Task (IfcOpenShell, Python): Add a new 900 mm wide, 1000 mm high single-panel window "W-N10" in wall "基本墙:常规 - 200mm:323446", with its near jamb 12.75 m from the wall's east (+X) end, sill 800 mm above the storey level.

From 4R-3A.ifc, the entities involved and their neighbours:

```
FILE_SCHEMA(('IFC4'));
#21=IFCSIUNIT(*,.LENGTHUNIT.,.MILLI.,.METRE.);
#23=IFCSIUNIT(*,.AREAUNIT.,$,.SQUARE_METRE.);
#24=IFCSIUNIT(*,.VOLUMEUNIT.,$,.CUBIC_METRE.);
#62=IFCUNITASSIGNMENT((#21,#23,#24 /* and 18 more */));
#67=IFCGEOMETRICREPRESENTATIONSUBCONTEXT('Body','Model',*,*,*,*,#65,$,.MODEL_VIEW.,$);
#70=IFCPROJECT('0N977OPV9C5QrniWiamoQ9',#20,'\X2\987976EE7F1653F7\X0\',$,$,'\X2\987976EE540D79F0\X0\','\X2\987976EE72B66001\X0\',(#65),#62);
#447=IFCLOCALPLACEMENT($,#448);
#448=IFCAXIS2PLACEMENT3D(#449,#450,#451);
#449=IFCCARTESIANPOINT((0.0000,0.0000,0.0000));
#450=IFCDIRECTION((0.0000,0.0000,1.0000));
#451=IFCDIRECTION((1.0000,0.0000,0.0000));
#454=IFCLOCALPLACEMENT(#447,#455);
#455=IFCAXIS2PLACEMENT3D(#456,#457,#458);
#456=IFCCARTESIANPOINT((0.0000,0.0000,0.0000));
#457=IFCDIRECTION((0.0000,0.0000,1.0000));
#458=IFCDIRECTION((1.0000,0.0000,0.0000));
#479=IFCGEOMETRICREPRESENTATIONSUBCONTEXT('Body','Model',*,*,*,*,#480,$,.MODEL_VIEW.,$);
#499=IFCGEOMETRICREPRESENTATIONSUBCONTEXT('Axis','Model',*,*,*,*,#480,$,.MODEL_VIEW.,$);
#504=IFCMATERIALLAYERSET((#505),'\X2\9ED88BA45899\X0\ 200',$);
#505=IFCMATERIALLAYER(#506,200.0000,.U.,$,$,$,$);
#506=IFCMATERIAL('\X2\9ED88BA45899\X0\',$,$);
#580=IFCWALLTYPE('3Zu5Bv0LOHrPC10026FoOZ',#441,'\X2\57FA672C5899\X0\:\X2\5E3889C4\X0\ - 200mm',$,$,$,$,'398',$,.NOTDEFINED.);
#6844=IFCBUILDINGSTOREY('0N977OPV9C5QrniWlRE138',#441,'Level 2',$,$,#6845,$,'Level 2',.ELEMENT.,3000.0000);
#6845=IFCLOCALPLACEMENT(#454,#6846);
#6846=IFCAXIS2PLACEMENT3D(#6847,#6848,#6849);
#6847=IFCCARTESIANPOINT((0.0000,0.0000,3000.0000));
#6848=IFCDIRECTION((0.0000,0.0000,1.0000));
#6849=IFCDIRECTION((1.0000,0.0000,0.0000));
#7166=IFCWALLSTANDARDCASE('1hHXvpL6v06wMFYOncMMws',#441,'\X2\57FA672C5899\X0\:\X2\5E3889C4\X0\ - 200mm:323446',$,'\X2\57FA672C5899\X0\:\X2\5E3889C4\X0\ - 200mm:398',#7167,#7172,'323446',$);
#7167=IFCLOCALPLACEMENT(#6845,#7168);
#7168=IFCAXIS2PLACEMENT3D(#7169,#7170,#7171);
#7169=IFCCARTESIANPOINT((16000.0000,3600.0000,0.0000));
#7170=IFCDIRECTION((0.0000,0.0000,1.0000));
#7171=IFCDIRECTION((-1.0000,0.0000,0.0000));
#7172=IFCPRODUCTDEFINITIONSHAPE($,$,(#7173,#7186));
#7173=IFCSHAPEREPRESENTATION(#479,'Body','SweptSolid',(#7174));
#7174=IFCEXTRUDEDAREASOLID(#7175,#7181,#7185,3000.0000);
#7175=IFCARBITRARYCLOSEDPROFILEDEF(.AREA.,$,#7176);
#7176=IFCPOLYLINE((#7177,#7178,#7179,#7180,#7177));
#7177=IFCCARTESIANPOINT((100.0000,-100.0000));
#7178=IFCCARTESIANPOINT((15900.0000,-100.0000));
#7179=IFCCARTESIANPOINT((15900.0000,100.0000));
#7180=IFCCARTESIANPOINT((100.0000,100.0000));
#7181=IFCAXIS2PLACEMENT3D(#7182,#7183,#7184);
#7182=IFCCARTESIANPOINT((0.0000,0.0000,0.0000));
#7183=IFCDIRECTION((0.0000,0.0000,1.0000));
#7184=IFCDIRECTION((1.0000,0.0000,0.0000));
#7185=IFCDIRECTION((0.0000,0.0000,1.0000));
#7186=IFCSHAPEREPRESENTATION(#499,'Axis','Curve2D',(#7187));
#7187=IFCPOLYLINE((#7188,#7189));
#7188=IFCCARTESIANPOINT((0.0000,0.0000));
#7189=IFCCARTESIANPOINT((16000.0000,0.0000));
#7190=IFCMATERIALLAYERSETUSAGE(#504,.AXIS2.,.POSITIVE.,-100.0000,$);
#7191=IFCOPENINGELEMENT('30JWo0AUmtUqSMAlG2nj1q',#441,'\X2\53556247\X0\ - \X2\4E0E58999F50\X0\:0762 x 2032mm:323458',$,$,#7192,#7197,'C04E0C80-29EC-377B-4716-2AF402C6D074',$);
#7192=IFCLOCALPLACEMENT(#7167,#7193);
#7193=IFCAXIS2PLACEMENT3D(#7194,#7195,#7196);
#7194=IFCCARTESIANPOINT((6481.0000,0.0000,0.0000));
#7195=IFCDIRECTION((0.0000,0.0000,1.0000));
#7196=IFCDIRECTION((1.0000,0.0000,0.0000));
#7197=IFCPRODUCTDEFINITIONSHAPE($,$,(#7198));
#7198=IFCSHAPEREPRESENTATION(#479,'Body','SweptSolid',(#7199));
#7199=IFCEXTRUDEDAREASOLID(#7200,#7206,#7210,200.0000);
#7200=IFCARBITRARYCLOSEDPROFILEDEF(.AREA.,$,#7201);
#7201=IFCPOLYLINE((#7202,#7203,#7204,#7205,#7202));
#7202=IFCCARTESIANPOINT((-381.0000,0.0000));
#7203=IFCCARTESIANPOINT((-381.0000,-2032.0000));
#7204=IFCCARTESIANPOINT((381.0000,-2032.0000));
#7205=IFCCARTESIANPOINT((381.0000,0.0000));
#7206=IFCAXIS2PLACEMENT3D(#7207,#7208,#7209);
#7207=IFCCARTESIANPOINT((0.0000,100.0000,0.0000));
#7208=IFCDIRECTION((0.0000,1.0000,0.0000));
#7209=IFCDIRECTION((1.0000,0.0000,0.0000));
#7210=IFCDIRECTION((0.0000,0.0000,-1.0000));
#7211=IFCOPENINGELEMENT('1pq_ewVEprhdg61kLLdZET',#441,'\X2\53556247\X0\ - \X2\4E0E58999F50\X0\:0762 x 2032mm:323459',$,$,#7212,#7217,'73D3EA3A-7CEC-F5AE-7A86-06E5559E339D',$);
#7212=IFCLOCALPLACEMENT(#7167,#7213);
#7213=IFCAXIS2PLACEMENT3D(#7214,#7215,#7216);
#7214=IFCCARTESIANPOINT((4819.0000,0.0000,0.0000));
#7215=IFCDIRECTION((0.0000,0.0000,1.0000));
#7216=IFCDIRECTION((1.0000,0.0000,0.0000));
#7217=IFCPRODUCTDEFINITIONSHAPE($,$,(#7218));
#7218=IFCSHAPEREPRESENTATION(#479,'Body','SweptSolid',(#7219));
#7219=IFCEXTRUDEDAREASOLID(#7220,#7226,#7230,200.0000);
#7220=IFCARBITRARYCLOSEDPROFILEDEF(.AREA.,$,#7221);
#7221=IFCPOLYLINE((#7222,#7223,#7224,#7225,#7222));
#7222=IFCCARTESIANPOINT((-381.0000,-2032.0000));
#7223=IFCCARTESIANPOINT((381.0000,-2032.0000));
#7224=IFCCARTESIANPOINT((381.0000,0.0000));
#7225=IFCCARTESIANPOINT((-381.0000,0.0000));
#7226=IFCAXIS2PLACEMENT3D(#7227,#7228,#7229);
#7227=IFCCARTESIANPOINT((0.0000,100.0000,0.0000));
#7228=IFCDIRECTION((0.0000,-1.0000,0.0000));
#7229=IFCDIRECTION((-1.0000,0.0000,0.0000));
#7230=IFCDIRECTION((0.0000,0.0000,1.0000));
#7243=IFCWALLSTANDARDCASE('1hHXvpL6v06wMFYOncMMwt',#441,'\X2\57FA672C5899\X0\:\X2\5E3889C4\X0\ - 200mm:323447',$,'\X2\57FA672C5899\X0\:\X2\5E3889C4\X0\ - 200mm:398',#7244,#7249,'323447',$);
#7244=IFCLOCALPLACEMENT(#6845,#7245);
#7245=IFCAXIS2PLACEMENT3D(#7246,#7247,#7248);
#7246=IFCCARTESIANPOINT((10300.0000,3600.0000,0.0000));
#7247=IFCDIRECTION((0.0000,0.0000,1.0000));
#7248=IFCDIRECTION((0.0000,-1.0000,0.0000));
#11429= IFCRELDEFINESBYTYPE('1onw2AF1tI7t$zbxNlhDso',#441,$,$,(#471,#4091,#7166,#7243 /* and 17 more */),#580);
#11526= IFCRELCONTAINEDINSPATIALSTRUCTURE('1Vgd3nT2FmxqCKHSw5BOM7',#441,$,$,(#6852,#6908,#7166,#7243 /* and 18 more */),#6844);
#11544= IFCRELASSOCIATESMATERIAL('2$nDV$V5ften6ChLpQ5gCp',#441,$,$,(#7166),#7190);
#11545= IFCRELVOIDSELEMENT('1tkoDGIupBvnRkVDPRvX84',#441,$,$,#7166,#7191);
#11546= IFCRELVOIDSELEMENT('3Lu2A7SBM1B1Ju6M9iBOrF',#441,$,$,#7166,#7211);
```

```python
import numpy as np
import ifcopenshell
import ifcopenshell.api.feature
import ifcopenshell.api.geometry
import ifcopenshell.api.root
import ifcopenshell.api.spatial
import ifcopenshell.geom
import ifcopenshell.util.element
import ifcopenshell.util.placement
import ifcopenshell.util.representation
import ifcopenshell.util.shape
import ifcopenshell.util.unit

model = ifcopenshell.open("4R-3A.ifc")
unit_scale = ifcopenshell.util.unit.calculate_unit_scale(model)
settings = ifcopenshell.geom.settings()


def volume(element):
    """Net volume in cubic metres, openings subtracted."""
    shape = ifcopenshell.geom.create_shape(settings, element)
    return ifcopenshell.util.shape.get_volume(shape.geometry)


wall = model.by_guid("1hHXvpL6v06wMFYOncMMws")
storey = ifcopenshell.util.element.get_container(wall, ifc_class="IfcBuildingStorey")
context = ifcopenshell.util.representation.get_context(model, "Model", "Body", "MODEL_VIEW")
before = volume(wall)

width, height, from_end, sill = 0.9, 1, 12.75, 0.8  # metres

# The wall runs along its own X axis, and the end named is its -X end.
wall_shape = ifcopenshell.geom.create_shape(settings, wall)
x, y, z = ifcopenshell.util.shape.get_vertices(wall_shape.geometry).T
start = x.min() + from_end
face, thickness = float(y.min()), float(y.max() - y.min())
wall_matrix = ifcopenshell.util.placement.get_local_placement(wall.ObjectPlacement)
level = ifcopenshell.util.placement.get_local_placement(storey.ObjectPlacement)[2, 3]


def in_wall(x, y):
    """Placement at x, y metres in the wall's axes, at sill height."""
    matrix = wall_matrix.copy()
    matrix[:, 3] = wall_matrix @ np.array([x / unit_scale, y / unit_scale, 0.0, 1.0])
    matrix[2, 3] = level + sill / unit_scale
    return matrix


# Opening: a box that overshoots both wall faces by 50 mm.
opening = ifcopenshell.api.root.create_entity(model, ifc_class="IfcOpeningElement", predefined_type="OPENING")
box = ifcopenshell.api.geometry.add_wall_representation(
    model, context=context, length=width, height=height, thickness=thickness + 0.1
)
ifcopenshell.api.geometry.assign_representation(model, product=opening, representation=box)
ifcopenshell.api.geometry.edit_object_placement(model, product=opening, matrix=in_wall(start, face - 0.05), is_si=False)
ifcopenshell.api.feature.add_feature(model, feature=opening, element=wall)

window = ifcopenshell.api.root.create_entity(model, ifc_class="IfcWindow", name="W-N10", predefined_type="WINDOW")
window.OverallWidth, window.OverallHeight = width / unit_scale, height / unit_scale
window.PartitioningType = "SINGLE_PANEL"
body = ifcopenshell.api.geometry.add_window_representation(
    model,
    context=context,
    overall_width=window.OverallWidth,
    overall_height=window.OverallHeight,
    partition_type="SINGLE_PANEL",
)
ifcopenshell.api.geometry.assign_representation(model, product=window, representation=body)
ifcopenshell.api.spatial.assign_container(model, products=[window], relating_structure=storey)
ifcopenshell.api.feature.add_filling(model, opening=opening, element=window)

# Centre the window in the wall's thickness.
ifcopenshell.api.geometry.edit_object_placement(model, product=window, matrix=in_wall(start, face), is_si=False)
window_shape = ifcopenshell.geom.create_shape(settings, window)
depth = ifcopenshell.util.shape.get_vertices(window_shape.geometry)[:, 1]
offset = face + thickness / 2 - (depth.min() + depth.max()) / 2
ifcopenshell.api.geometry.edit_object_placement(model, product=window, matrix=in_wall(start, offset), is_si=False)

after = volume(wall)

print(f"wall volume {before:.3f} -> {after:.3f} m3")

model.write("4R-3A-out.ifc")
```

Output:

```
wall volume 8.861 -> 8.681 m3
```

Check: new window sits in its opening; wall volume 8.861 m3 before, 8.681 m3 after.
